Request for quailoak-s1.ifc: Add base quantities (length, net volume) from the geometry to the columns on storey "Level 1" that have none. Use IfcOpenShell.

First a look at what the model holds.

```python
import ifcopenshell
import ifcopenshell.util.element
import ifcopenshell.util.unit

model = ifcopenshell.open("quailoak-s1.ifc")
print(model.schema)
for unit_type in ("LENGTHUNIT", "AREAUNIT", "VOLUMEUNIT"):
    print(unit_type, ifcopenshell.util.unit.calculate_unit_scale(model, unit_type))
storey = next(s for s in model.by_type("IfcBuildingStorey") if s.Name == "Level 1")
columns = [e for e in ifcopenshell.util.element.get_decomposition(storey) if e.is_a("IfcColumn")]
for e in sorted(columns, key=lambda e: e.id()):
    print(e.id(), e.is_a(), e.Name, list(ifcopenshell.util.element.get_psets(e, qtos_only=True)), sep=" | ")
```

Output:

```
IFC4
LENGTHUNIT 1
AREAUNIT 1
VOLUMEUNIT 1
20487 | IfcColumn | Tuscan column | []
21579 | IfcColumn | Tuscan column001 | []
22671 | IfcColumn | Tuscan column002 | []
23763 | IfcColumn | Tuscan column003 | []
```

```python
import ifcopenshell
import ifcopenshell.api.pset
import ifcopenshell.geom
import ifcopenshell.util.element
import ifcopenshell.util.shape
import ifcopenshell.util.unit

model = ifcopenshell.open("quailoak-s1.ifc")
unit_scale = ifcopenshell.util.unit.calculate_unit_scale(model)
volume_scale = ifcopenshell.util.unit.calculate_unit_scale(model, "VOLUMEUNIT")
settings = ifcopenshell.geom.settings()

storey = next(s for s in model.by_type("IfcBuildingStorey") if s.Name == "Level 1")
columns = [e for e in ifcopenshell.util.element.get_decomposition(storey) if e.is_a("IfcColumn")]

for e in sorted(columns, key=lambda e: e.id()):
    if ifcopenshell.util.element.get_psets(e, qtos_only=True, should_inherit=False):
        continue
    # Geometry comes back in metres, in the element's own axes.
    shape = ifcopenshell.geom.create_shape(settings, e)
    values = {
        "Length": ifcopenshell.util.shape.get_z(shape.geometry) / unit_scale,
        "NetVolume": ifcopenshell.util.shape.get_volume(shape.geometry) / volume_scale,
    }
    qto = ifcopenshell.api.pset.add_qto(model, product=e, name="Qto_ColumnBaseQuantities")
    ifcopenshell.api.pset.edit_qto(model, qto=qto, properties=values)
    print(e.id(), {k: round(v, 3) for k, v in values.items()})

model.write("quailoak-s1-out.ifc")
```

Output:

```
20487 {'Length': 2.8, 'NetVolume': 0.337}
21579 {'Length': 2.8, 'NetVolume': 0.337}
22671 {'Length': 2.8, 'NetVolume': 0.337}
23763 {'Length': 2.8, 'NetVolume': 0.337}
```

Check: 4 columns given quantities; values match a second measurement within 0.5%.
